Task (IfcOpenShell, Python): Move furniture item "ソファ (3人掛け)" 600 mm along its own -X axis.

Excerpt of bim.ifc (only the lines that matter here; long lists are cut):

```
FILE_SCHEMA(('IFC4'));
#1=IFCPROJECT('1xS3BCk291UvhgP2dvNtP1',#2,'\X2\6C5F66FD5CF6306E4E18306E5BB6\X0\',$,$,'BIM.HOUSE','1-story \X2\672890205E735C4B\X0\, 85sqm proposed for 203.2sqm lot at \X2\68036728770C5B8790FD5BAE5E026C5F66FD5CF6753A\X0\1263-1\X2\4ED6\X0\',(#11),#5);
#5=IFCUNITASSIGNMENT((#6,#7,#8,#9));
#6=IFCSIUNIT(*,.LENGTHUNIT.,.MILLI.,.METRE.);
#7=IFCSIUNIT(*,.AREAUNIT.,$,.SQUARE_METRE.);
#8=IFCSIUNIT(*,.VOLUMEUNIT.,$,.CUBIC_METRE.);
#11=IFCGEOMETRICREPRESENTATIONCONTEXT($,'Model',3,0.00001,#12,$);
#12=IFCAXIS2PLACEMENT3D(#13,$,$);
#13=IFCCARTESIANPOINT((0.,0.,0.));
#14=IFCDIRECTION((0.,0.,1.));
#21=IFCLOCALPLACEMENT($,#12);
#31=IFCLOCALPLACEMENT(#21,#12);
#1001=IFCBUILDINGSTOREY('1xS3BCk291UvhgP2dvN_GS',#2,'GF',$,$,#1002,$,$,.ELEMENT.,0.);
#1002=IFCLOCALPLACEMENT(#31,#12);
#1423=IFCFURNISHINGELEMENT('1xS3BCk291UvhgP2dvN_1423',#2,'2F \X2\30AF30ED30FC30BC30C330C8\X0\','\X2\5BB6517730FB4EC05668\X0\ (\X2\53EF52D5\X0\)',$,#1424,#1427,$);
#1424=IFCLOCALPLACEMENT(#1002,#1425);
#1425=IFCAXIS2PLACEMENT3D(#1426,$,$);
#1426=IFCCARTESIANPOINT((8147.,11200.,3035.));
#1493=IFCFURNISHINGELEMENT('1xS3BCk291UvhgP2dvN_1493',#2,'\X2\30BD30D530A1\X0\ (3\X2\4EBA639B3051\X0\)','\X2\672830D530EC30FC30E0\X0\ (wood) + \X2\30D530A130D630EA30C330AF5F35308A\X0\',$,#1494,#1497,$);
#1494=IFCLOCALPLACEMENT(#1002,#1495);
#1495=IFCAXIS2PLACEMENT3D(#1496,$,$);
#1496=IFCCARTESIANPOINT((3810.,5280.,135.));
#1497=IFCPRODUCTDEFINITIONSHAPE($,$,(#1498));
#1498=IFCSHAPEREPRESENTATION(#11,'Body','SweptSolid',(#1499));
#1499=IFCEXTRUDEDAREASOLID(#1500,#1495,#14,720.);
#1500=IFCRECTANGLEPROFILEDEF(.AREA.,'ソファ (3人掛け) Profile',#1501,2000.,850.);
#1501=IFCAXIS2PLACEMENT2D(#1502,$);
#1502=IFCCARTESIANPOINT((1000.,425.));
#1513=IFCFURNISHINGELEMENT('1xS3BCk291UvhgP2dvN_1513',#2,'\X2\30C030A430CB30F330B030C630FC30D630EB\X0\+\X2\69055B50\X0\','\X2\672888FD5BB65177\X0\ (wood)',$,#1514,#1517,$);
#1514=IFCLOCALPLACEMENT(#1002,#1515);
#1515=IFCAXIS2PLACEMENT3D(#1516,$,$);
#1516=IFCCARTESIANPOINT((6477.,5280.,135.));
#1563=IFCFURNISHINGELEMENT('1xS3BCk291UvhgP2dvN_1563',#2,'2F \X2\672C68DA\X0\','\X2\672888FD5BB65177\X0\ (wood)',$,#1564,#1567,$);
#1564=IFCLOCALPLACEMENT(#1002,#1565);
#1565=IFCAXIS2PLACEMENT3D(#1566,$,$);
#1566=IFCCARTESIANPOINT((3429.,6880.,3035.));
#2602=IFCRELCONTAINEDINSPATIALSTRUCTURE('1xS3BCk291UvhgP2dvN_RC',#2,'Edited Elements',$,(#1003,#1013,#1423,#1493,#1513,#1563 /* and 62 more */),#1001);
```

```python
import ifcopenshell
import ifcopenshell.api.geometry
import ifcopenshell.util.placement

model = ifcopenshell.open("bim.ifc")

item = model.by_guid("1xS3BCk291UvhgP2dvN_1493")
matrix = ifcopenshell.util.placement.get_local_placement(item.ObjectPlacement)
matrix[:3, 3] -= matrix[:3, 0] * 600.0
ifcopenshell.api.geometry.edit_object_placement(model, product=item, matrix=matrix, is_si=False)

print(ifcopenshell.util.placement.get_local_placement(item.ObjectPlacement).round(3) + 0.0)

model.write("bim_edited.ifc")
```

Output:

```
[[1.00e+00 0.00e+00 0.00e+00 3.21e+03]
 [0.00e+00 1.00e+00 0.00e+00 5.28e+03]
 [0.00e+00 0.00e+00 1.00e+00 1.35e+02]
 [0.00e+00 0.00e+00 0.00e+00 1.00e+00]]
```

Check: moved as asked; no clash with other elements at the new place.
